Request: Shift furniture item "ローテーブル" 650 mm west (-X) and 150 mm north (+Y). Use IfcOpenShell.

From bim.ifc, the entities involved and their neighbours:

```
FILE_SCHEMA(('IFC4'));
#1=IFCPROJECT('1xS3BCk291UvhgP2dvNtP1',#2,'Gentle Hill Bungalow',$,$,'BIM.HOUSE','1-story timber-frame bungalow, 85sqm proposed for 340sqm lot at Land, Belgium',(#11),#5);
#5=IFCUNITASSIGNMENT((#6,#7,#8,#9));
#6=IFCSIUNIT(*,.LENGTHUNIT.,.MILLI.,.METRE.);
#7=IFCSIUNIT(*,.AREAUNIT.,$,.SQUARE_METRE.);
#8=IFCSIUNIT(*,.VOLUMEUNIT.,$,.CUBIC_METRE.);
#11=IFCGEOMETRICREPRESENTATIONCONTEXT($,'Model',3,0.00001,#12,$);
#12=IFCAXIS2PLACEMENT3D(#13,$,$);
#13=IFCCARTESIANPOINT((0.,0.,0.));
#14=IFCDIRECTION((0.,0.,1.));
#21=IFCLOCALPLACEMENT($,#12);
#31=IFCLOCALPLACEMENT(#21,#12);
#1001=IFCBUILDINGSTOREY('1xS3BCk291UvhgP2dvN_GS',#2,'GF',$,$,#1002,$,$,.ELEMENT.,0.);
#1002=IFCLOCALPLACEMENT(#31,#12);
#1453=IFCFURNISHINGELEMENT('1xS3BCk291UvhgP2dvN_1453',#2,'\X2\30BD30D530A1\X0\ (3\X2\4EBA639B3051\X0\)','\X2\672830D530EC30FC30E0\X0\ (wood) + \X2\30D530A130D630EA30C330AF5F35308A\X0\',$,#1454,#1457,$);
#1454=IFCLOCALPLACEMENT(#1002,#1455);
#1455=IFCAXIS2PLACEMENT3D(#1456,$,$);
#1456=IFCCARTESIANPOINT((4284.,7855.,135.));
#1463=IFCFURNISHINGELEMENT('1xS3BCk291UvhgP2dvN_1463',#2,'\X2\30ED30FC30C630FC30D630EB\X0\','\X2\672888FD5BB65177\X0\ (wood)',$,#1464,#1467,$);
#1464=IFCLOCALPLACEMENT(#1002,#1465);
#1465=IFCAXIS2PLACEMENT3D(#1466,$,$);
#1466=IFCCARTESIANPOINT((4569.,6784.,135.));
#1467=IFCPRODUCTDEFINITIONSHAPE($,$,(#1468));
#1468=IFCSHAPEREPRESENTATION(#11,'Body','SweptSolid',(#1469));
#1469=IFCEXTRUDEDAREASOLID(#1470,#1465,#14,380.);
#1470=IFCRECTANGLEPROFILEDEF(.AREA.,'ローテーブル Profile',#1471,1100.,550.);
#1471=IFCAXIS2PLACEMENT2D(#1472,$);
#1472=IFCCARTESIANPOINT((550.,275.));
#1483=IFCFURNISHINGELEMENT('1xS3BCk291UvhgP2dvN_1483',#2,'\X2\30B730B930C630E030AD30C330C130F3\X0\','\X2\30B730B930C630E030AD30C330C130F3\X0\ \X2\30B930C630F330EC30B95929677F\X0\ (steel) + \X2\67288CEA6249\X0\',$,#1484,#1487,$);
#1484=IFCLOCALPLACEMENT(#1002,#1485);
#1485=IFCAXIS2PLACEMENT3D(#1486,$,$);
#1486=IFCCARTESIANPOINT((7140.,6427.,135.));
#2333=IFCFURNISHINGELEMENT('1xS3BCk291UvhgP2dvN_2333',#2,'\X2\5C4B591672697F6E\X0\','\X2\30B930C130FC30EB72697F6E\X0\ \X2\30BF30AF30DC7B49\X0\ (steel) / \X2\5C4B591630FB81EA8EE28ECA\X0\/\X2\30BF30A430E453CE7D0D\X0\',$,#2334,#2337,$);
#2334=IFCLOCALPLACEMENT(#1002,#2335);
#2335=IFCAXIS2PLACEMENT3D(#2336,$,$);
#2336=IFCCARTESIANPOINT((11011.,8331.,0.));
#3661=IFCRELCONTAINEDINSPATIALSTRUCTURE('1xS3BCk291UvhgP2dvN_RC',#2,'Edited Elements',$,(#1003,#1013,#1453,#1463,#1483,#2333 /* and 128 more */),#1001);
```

```python
import ifcopenshell
import ifcopenshell.api.geometry
import ifcopenshell.util.placement

model = ifcopenshell.open("bim.ifc")

item = model.by_guid("1xS3BCk291UvhgP2dvN_1463")
matrix = ifcopenshell.util.placement.get_local_placement(item.ObjectPlacement)
matrix[0, 3] -= 650.0
matrix[1, 3] += 150.0
ifcopenshell.api.geometry.edit_object_placement(model, product=item, matrix=matrix, is_si=False)

print(ifcopenshell.util.placement.get_local_placement(item.ObjectPlacement).round(3) + 0.0)

model.write("bim_rev.ifc")
```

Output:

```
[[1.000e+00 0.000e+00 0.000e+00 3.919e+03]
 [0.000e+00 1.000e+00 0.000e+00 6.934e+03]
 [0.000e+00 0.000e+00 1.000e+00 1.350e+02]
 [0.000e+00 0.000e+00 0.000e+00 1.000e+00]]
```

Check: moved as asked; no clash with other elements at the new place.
